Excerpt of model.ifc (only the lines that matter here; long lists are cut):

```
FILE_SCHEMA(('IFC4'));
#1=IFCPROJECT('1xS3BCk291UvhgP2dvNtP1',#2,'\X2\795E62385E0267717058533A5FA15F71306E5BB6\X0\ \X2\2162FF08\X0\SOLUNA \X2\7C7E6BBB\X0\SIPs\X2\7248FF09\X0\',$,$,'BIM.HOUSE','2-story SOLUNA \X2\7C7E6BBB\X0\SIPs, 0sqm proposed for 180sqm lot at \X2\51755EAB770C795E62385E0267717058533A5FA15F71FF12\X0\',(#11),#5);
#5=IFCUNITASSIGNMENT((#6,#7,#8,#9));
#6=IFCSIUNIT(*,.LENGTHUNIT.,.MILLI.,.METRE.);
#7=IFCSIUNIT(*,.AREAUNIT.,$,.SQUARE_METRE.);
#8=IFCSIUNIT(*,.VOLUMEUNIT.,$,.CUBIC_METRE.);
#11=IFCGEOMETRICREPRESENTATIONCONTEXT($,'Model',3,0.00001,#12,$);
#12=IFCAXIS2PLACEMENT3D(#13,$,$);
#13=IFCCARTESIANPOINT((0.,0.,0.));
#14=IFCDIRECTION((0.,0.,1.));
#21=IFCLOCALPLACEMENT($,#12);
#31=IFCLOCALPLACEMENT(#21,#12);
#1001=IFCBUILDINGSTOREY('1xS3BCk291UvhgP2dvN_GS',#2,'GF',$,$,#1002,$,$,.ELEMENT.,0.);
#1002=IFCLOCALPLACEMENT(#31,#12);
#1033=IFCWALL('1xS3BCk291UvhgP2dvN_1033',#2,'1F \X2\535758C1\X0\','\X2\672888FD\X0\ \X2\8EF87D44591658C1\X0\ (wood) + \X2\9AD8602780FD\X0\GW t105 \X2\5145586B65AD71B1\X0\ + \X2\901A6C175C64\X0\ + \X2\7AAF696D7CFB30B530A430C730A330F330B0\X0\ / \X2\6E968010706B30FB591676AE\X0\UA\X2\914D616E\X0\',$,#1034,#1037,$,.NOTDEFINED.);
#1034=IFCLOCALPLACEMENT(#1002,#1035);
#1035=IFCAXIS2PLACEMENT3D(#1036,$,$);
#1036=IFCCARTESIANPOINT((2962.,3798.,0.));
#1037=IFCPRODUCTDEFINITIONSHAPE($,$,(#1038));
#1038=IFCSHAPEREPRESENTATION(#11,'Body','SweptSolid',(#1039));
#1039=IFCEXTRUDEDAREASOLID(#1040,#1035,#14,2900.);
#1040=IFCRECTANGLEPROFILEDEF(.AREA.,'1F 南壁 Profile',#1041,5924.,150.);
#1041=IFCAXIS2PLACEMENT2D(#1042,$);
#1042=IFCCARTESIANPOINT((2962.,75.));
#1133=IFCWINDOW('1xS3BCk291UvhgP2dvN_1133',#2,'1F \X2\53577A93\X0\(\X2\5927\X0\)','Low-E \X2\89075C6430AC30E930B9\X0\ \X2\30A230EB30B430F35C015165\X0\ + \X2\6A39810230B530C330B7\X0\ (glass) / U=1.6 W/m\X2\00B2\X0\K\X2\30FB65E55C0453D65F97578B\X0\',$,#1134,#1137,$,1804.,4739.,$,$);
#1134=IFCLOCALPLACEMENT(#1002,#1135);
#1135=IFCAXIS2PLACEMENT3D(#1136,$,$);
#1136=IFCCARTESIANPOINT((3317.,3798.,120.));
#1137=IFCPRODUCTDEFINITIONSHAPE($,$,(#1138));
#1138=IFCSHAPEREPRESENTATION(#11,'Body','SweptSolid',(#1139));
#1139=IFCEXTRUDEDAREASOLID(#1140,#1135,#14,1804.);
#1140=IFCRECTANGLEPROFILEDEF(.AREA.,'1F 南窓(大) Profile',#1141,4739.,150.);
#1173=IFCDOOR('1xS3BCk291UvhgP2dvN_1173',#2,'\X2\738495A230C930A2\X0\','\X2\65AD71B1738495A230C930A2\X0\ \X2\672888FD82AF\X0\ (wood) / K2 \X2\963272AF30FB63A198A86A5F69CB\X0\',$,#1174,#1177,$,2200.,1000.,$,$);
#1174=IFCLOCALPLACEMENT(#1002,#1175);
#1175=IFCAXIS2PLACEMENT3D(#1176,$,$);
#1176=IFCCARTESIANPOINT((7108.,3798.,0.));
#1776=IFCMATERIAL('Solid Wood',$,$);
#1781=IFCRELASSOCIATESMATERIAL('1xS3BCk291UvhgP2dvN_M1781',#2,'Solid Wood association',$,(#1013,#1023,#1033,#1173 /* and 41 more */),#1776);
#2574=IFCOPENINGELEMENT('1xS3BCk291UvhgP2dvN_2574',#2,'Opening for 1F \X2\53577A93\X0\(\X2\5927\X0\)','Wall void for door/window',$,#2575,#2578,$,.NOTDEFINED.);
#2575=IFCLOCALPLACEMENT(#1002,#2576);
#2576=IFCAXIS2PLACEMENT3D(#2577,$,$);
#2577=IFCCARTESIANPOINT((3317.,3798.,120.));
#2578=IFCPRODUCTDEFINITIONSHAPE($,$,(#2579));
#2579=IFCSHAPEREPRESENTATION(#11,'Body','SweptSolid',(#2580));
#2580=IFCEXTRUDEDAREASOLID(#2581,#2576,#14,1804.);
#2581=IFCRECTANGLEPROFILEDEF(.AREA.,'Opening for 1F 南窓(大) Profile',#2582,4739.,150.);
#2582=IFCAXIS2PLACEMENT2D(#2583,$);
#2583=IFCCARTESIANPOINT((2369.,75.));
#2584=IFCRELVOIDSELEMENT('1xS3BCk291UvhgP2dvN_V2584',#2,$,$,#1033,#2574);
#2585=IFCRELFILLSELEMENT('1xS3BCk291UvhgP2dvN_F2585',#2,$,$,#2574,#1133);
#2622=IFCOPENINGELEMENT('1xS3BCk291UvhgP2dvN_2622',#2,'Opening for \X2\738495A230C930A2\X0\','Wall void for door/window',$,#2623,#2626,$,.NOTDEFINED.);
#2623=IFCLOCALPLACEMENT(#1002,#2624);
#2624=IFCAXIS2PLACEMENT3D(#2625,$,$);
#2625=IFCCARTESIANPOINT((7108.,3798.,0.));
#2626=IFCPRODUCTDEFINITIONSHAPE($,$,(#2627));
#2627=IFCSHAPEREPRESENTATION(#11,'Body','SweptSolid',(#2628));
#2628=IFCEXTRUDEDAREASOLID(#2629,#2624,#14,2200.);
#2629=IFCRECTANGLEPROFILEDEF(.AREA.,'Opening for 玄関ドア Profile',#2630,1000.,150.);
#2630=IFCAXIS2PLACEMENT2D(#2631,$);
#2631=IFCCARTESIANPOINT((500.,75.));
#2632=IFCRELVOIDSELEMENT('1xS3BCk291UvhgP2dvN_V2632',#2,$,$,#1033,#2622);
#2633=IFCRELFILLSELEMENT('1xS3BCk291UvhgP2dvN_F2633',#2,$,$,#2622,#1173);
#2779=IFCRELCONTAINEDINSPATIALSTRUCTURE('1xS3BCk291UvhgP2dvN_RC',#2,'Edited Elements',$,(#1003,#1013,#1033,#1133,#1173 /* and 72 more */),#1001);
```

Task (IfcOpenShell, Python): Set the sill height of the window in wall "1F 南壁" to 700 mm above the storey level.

```python
import numpy as np
import ifcopenshell
import ifcopenshell.api.geometry
import ifcopenshell.geom
import ifcopenshell.util.element
import ifcopenshell.util.placement
import ifcopenshell.util.shape
import ifcopenshell.util.unit

model = ifcopenshell.open("model.ifc")
unit_scale = ifcopenshell.util.unit.calculate_unit_scale(model)

window = model.by_id(1133)
opening = window.FillsVoids[0].RelatingOpeningElement
storey = ifcopenshell.util.element.get_container(window, ifc_class="IfcBuildingStorey")
level = ifcopenshell.util.placement.get_local_placement(storey.ObjectPlacement)[2, 3]

# The opening's origin need not be at the sill, so measure its lowest point.
shape = ifcopenshell.geom.create_shape(ifcopenshell.geom.settings(), opening)
bottom = ifcopenshell.util.shape.get_shape_bottom_elevation(shape, shape.geometry) / unit_scale
dz = level + 700.0 - bottom

shift = np.array([0.0, 0.0, dz])
# The window is not placed relative to its opening, so move both.
for product in (opening, window):
    matrix = ifcopenshell.util.placement.get_local_placement(product.ObjectPlacement)
    matrix[:3, 3] += shift
    ifcopenshell.api.geometry.edit_object_placement(model, product=product, matrix=matrix, is_si=False)

print(f"moved by {dz * unit_scale:+.3f} m")

model.write("model_updated.ifc")
```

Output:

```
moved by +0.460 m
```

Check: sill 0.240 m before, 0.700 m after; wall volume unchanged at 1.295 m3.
